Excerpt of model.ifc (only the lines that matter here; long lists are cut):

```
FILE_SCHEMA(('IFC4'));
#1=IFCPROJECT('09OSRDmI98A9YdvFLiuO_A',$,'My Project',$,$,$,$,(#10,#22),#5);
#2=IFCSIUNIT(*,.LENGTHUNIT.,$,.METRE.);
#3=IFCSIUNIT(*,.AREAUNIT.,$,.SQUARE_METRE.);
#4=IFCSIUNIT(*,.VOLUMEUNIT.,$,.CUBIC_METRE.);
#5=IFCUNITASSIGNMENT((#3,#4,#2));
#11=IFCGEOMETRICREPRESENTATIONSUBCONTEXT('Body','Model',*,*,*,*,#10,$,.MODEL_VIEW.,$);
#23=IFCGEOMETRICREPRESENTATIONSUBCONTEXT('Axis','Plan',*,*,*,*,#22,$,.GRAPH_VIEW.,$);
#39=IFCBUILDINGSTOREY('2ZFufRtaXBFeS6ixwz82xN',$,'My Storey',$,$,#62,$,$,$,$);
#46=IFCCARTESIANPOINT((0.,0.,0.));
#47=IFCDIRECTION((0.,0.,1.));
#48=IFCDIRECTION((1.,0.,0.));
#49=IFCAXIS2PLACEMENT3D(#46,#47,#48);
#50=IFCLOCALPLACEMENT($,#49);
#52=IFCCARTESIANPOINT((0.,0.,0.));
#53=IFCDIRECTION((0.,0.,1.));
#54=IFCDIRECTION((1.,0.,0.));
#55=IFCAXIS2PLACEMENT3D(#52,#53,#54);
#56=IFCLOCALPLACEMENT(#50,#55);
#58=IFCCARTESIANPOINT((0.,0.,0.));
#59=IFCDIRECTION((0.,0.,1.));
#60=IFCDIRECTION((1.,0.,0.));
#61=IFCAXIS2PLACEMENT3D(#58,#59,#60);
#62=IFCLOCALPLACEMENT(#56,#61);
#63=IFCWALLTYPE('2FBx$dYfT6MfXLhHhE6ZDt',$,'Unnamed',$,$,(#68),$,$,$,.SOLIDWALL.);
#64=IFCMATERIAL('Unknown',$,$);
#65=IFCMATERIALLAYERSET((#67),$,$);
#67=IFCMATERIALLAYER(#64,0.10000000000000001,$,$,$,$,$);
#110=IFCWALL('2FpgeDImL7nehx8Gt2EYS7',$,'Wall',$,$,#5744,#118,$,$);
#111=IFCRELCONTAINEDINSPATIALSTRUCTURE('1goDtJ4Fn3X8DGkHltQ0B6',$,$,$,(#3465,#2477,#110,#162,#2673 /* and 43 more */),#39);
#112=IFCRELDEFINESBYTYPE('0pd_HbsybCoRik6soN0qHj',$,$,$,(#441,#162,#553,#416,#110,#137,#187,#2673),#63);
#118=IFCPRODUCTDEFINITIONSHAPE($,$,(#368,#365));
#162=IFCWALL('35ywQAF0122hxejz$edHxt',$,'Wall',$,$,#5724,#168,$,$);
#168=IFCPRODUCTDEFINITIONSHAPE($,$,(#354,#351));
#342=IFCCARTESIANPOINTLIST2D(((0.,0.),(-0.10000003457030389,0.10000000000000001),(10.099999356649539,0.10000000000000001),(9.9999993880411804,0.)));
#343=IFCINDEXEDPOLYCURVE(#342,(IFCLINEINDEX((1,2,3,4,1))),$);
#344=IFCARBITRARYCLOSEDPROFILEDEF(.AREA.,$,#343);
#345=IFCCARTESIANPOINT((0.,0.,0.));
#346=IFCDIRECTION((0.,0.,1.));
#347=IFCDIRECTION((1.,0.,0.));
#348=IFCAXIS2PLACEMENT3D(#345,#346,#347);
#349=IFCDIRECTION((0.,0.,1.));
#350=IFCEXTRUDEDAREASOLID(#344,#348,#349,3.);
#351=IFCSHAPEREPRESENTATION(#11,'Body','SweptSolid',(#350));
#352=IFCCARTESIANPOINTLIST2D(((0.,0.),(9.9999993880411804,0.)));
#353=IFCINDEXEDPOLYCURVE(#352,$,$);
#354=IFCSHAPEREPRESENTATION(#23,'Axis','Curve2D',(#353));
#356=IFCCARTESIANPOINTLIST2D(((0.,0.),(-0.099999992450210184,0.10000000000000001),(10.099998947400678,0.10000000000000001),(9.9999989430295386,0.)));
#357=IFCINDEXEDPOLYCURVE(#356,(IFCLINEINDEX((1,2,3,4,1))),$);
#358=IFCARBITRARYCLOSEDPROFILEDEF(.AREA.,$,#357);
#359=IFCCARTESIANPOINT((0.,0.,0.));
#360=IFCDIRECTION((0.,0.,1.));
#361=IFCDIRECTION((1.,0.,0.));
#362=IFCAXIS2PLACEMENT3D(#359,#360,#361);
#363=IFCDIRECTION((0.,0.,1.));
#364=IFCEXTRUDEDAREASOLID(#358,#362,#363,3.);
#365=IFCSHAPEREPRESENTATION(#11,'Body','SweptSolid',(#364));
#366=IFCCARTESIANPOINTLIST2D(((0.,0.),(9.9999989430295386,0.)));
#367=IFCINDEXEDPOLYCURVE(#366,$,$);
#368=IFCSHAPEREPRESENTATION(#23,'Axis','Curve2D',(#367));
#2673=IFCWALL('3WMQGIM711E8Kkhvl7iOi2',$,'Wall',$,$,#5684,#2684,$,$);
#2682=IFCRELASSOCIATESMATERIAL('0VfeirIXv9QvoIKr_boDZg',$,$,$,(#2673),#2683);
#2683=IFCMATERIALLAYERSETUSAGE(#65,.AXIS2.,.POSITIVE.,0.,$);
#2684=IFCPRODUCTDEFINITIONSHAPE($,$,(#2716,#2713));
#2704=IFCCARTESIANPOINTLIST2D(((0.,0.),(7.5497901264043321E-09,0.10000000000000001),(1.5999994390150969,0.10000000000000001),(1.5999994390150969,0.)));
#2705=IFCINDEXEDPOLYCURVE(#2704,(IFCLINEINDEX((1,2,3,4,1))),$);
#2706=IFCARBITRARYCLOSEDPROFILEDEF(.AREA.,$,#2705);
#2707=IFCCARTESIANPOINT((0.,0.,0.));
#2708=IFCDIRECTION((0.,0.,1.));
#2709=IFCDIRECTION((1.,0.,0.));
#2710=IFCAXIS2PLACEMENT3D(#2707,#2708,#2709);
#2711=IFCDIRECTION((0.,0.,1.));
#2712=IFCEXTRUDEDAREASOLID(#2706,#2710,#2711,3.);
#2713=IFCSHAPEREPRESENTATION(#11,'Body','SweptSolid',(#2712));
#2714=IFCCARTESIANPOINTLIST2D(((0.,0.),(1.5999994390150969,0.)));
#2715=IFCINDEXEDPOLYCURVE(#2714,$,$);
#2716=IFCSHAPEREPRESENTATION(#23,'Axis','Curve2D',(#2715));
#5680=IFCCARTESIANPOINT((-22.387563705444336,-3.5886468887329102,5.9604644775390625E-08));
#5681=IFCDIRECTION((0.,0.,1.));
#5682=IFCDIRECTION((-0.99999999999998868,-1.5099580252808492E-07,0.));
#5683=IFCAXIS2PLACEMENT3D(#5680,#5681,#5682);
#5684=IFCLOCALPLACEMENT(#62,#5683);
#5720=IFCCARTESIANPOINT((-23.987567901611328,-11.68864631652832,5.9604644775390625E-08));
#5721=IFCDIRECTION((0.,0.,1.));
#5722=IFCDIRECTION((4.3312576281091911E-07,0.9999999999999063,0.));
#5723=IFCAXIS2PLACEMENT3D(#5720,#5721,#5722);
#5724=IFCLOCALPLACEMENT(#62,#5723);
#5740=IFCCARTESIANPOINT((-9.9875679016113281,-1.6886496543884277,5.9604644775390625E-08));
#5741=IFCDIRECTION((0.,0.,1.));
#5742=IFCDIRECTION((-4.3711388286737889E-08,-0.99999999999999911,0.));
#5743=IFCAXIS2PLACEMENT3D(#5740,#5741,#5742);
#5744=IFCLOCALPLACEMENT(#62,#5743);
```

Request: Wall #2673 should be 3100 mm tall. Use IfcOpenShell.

```python
import ifcopenshell
import ifcopenshell.geom
import ifcopenshell.util.representation
import ifcopenshell.util.shape

model = ifcopenshell.open("model.ifc")
settings = ifcopenshell.geom.settings()


def volume(element):
    """Net volume in cubic metres, openings subtracted."""
    shape = ifcopenshell.geom.create_shape(settings, element)
    return ifcopenshell.util.shape.get_volume(shape.geometry)


wall = model.by_guid("3WMQGIM711E8Kkhvl7iOi2")
before = volume(wall)

body = ifcopenshell.util.representation.get_representation(wall, "Model", "Body")
solid = body.Items[0]
old_height = solid.Depth
solid.Depth = 3.1
after = volume(wall)

print(f"height {old_height:g} -> {solid.Depth:g}, volume {before:.3f} -> {after:.3f} m3")

model.write("model-out.ifc")
```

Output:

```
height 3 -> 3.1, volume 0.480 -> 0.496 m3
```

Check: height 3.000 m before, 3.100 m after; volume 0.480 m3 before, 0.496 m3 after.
